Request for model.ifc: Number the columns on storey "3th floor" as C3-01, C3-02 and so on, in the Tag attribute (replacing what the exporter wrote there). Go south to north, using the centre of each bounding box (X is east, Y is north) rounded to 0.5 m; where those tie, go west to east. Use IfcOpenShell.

First a look at what the model holds.

```python
import ifcopenshell
import ifcopenshell.util.element
import ifcopenshell.util.placement

model = ifcopenshell.open("model.ifc")
print(model.schema)
storey = next(s for s in model.by_type("IfcBuildingStorey") if s.Name == "3th floor")
columns = [e for e in ifcopenshell.util.element.get_decomposition(storey) if e.is_a("IfcColumn")]
for e in sorted(columns, key=lambda e: e.id()):
    origin = ifcopenshell.util.placement.get_local_placement(e.ObjectPlacement)[:3, 3]
    print(e.id(), e.Tag, e.Name, origin.round(2) + 0.0, sep=" | ")
```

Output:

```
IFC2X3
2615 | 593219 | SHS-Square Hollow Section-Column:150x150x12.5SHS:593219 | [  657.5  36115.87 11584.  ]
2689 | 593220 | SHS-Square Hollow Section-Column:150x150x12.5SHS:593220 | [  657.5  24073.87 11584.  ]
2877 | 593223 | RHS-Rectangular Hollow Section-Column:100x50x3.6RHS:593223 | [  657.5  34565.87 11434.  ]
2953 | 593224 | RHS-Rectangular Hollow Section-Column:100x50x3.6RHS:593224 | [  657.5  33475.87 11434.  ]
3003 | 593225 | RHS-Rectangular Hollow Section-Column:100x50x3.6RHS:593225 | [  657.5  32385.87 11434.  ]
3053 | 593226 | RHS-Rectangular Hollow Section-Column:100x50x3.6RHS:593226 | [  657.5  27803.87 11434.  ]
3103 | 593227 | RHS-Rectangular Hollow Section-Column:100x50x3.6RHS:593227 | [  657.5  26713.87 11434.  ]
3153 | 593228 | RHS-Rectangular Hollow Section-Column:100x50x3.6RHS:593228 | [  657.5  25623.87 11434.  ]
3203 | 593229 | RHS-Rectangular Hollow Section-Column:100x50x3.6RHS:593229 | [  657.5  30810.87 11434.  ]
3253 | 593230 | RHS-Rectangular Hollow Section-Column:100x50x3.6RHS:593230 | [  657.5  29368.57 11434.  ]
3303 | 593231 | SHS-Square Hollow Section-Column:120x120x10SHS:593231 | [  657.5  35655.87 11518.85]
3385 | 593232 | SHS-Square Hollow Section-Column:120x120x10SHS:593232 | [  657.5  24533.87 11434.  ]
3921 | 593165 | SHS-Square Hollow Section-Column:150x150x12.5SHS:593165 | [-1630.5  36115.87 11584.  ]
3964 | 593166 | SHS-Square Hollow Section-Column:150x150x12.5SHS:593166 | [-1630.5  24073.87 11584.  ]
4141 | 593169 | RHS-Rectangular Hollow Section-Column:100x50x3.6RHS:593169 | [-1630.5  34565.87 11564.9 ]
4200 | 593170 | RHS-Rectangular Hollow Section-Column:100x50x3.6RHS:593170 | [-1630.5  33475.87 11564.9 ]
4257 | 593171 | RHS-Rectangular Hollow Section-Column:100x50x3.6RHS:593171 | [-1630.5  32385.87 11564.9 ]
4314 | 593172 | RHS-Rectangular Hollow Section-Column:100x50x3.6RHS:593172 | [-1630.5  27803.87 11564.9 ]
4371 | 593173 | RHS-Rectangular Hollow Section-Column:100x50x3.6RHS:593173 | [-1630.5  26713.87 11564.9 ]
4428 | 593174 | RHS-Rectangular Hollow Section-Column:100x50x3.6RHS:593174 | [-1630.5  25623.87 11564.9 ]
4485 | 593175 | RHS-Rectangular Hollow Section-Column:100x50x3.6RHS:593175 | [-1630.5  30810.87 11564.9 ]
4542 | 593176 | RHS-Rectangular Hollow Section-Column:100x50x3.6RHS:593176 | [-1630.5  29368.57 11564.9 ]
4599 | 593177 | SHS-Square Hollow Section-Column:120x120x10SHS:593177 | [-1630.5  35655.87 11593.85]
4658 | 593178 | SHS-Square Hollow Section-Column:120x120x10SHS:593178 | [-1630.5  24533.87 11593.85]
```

```python
import ifcopenshell
import ifcopenshell.geom
import ifcopenshell.util.element
import ifcopenshell.util.shape

model = ifcopenshell.open("model.ifc")
settings = ifcopenshell.geom.settings()
settings.set("use-world-coords", True)


def centre(element):
    shape = ifcopenshell.geom.create_shape(settings, element)
    return ifcopenshell.util.shape.get_bbox_centroid(shape.geometry)


storey = next(s for s in model.by_type("IfcBuildingStorey") if s.Name == "3th floor")
columns = [e for e in ifcopenshell.util.element.get_decomposition(storey) if e.is_a("IfcColumn")]

# Insertion points can sit at a corner or the storey origin, so sort by the geometry (in metres).
centres = {e: centre(e) for e in columns}
columns.sort(key=lambda e: (round(centres[e][1] / 0.5), centres[e][0]))

for i, e in enumerate(columns, start=1):
    number = f"C3-{i:02d}"
    e.Tag = number
    print(e.id(), number)

model.write("model_edited.ifc")
```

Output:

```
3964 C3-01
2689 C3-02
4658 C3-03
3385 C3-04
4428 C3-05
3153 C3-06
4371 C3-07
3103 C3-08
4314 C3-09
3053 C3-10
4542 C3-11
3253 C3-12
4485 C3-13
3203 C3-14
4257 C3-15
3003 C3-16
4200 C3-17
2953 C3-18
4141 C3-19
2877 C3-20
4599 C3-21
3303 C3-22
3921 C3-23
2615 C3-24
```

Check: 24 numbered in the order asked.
